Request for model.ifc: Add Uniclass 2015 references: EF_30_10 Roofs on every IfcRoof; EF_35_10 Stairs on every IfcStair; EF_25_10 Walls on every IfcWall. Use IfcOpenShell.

First a look at what the model holds.

```python
import ifcopenshell

model = ifcopenshell.open("model.ifc")
print(model.schema)
print("classifications:", [c.Name for c in model.by_type("IfcClassification")])
for ifc_class in ("IfcDoor", "IfcRoof", "IfcStair", "IfcWall", "IfcWindow"):
    print(ifc_class, len(model.by_type(ifc_class)))
```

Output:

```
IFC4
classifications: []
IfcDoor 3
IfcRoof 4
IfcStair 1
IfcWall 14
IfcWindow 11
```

```python
import ifcopenshell
import ifcopenshell.api.classification

model = ifcopenshell.open("model.ifc")

system = ifcopenshell.api.classification.add_classification(model, classification="Uniclass 2015")

codes = {
    "IfcRoof": ("EF_30_10", "Roofs"),
    "IfcStair": ("EF_35_10", "Stairs"),
    "IfcWall": ("EF_25_10", "Walls"),
}
for ifc_class, (code, name) in codes.items():
    products = model.by_type(ifc_class)
    ifcopenshell.api.classification.add_reference(
        model, products=products, classification=system, identification=code, name=name
    )
    print(code, len(products))

model.write("model_v2.ifc")
```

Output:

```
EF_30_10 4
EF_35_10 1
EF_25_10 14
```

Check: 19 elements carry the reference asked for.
